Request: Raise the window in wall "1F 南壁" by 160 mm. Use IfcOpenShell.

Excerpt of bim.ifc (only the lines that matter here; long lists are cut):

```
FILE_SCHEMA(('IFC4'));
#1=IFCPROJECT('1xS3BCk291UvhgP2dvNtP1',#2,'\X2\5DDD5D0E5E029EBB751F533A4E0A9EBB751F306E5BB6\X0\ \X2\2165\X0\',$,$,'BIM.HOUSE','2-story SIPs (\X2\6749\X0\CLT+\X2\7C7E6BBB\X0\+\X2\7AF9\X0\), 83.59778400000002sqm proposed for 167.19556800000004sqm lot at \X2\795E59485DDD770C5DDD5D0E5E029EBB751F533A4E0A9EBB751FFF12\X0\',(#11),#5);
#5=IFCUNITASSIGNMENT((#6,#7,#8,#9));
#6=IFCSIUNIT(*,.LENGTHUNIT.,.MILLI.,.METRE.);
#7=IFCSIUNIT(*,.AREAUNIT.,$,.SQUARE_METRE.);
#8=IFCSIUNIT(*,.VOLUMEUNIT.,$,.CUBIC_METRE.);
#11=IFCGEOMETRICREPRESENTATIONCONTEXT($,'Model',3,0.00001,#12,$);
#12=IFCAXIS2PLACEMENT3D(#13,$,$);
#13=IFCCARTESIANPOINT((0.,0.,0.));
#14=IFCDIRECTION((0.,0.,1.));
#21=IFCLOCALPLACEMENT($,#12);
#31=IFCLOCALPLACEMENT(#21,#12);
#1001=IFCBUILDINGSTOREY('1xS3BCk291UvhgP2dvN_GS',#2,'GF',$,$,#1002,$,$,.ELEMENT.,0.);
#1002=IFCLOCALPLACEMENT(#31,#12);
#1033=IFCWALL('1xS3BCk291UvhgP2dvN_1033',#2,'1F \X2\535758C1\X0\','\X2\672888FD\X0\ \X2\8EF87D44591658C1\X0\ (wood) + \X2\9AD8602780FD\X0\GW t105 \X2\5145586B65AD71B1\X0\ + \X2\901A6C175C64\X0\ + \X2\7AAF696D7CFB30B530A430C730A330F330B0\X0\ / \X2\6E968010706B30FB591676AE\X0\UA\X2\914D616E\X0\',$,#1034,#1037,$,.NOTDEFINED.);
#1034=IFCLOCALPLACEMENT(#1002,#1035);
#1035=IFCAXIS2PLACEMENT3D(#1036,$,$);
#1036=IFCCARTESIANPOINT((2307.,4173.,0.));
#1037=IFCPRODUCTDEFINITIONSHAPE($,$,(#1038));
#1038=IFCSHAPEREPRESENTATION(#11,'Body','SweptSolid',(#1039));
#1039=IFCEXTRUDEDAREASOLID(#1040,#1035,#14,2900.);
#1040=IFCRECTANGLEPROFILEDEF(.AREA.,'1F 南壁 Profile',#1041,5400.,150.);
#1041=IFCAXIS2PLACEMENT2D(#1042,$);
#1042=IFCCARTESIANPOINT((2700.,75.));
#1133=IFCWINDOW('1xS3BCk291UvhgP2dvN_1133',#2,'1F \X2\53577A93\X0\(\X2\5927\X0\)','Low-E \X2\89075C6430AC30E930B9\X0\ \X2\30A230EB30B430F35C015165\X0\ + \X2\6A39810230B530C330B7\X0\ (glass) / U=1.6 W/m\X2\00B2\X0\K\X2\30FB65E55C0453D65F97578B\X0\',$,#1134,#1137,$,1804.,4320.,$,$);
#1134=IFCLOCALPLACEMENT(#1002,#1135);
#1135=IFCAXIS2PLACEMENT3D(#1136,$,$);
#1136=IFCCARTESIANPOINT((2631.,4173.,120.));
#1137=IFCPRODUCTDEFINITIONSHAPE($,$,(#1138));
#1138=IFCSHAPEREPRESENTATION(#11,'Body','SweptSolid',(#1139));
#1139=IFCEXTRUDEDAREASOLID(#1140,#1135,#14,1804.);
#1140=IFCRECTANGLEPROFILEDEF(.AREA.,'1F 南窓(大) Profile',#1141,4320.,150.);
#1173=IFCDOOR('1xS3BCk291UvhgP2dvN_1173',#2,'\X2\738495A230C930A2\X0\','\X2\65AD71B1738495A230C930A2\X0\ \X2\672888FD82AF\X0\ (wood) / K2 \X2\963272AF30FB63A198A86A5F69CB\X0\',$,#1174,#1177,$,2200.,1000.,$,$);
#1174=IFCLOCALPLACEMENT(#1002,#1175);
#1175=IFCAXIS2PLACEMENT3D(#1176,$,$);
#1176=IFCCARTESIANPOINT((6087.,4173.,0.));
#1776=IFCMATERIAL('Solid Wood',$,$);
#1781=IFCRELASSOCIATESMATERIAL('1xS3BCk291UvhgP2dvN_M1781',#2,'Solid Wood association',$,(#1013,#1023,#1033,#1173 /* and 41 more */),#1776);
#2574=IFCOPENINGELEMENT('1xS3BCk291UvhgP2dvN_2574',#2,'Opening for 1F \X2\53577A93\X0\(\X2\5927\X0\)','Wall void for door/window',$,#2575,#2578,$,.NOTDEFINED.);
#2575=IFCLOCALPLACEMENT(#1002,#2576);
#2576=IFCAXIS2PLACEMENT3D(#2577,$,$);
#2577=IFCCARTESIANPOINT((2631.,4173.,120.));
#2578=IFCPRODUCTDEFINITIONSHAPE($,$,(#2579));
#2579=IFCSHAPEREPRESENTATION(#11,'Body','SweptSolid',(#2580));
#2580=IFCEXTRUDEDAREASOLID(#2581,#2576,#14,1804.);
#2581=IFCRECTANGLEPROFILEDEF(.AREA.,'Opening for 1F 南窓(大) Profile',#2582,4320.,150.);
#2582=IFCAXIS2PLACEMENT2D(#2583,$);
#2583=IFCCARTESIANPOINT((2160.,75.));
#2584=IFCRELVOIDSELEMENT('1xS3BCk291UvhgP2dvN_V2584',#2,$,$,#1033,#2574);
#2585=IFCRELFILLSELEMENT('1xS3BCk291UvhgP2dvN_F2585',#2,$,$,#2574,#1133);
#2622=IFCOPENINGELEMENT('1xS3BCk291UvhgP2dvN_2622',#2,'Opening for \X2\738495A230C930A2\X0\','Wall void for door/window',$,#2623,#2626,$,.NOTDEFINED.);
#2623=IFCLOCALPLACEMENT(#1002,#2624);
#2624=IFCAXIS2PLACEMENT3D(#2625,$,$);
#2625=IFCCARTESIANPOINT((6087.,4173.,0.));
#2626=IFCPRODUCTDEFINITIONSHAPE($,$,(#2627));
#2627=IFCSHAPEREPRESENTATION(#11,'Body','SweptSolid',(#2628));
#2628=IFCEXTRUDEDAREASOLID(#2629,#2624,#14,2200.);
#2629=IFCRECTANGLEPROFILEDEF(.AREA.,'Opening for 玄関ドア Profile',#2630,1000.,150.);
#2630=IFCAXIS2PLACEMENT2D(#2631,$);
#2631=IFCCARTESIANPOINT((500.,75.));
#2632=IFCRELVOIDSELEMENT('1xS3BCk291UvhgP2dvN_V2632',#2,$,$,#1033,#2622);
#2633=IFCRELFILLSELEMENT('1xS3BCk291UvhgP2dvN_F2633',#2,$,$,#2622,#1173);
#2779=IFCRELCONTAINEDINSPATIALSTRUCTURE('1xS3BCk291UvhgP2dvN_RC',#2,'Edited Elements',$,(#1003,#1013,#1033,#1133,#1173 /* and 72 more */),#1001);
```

```python
import numpy as np
import ifcopenshell
import ifcopenshell.api.geometry
import ifcopenshell.util.placement
import ifcopenshell.util.unit

model = ifcopenshell.open("bim.ifc")
unit_scale = ifcopenshell.util.unit.calculate_unit_scale(model)

window = model.by_guid("1xS3BCk291UvhgP2dvN_1133")
opening = window.FillsVoids[0].RelatingOpeningElement
dz = 0.16 / unit_scale

shift = np.array([0.0, 0.0, dz])
# The window is not placed relative to its opening, so move both.
for product in (opening, window):
    matrix = ifcopenshell.util.placement.get_local_placement(product.ObjectPlacement)
    matrix[:3, 3] += shift
    ifcopenshell.api.geometry.edit_object_placement(model, product=product, matrix=matrix, is_si=False)

print(f"moved by {dz * unit_scale:+.3f} m")

model.write("bim_v2.ifc")
```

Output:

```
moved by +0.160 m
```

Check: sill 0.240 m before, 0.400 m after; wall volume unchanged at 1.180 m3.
